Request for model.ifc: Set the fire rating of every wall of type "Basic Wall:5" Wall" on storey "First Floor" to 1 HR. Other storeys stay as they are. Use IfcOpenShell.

First a look at what the model holds.

```python
import ifcopenshell
import ifcopenshell.util.element

model = ifcopenshell.open("model.ifc")
print(model.schema)
storey = next(s for s in model.by_type("IfcBuildingStorey") if s.Name == "First Floor")
walls = [e for e in ifcopenshell.util.element.get_decomposition(storey) if e.is_a("IfcWall")]
seen = {}
for e in walls:
    element_type = ifcopenshell.util.element.get_type(e)
    key = (element_type.Name if element_type != e and element_type else None, ifcopenshell.util.element.get_pset(e, "Pset_WallCommon", "FireRating"))
    seen[key] = seen.get(key, 0) + 1
for (name, value), count in sorted(seen.items(), key=str):
    print(count, "x", name, "|", value)
```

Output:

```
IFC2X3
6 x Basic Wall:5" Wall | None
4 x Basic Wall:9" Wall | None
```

```python
import ifcopenshell
import ifcopenshell.api.pset
import ifcopenshell.util.element

model = ifcopenshell.open("model.ifc")

storey = next(s for s in model.by_type("IfcBuildingStorey") if s.Name == "First Floor")
walls = [e for e in ifcopenshell.util.element.get_decomposition(storey) if e.is_a("IfcWall")]

count = 0
for e in walls:
    element_type = ifcopenshell.util.element.get_type(e)
    if element_type in (None, e) or element_type.Name != 'Basic Wall:5" Wall':
        continue
    # add_pset returns the element's existing set when there is one.
    pset = ifcopenshell.api.pset.add_pset(model, product=e, name="Pset_WallCommon")
    ifcopenshell.api.pset.edit_pset(model, pset=pset, properties={"FireRating": "1 HR"})
    count += 1

print(count, "walls updated")

model.write("model_v2.ifc")
```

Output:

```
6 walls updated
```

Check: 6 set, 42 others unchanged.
